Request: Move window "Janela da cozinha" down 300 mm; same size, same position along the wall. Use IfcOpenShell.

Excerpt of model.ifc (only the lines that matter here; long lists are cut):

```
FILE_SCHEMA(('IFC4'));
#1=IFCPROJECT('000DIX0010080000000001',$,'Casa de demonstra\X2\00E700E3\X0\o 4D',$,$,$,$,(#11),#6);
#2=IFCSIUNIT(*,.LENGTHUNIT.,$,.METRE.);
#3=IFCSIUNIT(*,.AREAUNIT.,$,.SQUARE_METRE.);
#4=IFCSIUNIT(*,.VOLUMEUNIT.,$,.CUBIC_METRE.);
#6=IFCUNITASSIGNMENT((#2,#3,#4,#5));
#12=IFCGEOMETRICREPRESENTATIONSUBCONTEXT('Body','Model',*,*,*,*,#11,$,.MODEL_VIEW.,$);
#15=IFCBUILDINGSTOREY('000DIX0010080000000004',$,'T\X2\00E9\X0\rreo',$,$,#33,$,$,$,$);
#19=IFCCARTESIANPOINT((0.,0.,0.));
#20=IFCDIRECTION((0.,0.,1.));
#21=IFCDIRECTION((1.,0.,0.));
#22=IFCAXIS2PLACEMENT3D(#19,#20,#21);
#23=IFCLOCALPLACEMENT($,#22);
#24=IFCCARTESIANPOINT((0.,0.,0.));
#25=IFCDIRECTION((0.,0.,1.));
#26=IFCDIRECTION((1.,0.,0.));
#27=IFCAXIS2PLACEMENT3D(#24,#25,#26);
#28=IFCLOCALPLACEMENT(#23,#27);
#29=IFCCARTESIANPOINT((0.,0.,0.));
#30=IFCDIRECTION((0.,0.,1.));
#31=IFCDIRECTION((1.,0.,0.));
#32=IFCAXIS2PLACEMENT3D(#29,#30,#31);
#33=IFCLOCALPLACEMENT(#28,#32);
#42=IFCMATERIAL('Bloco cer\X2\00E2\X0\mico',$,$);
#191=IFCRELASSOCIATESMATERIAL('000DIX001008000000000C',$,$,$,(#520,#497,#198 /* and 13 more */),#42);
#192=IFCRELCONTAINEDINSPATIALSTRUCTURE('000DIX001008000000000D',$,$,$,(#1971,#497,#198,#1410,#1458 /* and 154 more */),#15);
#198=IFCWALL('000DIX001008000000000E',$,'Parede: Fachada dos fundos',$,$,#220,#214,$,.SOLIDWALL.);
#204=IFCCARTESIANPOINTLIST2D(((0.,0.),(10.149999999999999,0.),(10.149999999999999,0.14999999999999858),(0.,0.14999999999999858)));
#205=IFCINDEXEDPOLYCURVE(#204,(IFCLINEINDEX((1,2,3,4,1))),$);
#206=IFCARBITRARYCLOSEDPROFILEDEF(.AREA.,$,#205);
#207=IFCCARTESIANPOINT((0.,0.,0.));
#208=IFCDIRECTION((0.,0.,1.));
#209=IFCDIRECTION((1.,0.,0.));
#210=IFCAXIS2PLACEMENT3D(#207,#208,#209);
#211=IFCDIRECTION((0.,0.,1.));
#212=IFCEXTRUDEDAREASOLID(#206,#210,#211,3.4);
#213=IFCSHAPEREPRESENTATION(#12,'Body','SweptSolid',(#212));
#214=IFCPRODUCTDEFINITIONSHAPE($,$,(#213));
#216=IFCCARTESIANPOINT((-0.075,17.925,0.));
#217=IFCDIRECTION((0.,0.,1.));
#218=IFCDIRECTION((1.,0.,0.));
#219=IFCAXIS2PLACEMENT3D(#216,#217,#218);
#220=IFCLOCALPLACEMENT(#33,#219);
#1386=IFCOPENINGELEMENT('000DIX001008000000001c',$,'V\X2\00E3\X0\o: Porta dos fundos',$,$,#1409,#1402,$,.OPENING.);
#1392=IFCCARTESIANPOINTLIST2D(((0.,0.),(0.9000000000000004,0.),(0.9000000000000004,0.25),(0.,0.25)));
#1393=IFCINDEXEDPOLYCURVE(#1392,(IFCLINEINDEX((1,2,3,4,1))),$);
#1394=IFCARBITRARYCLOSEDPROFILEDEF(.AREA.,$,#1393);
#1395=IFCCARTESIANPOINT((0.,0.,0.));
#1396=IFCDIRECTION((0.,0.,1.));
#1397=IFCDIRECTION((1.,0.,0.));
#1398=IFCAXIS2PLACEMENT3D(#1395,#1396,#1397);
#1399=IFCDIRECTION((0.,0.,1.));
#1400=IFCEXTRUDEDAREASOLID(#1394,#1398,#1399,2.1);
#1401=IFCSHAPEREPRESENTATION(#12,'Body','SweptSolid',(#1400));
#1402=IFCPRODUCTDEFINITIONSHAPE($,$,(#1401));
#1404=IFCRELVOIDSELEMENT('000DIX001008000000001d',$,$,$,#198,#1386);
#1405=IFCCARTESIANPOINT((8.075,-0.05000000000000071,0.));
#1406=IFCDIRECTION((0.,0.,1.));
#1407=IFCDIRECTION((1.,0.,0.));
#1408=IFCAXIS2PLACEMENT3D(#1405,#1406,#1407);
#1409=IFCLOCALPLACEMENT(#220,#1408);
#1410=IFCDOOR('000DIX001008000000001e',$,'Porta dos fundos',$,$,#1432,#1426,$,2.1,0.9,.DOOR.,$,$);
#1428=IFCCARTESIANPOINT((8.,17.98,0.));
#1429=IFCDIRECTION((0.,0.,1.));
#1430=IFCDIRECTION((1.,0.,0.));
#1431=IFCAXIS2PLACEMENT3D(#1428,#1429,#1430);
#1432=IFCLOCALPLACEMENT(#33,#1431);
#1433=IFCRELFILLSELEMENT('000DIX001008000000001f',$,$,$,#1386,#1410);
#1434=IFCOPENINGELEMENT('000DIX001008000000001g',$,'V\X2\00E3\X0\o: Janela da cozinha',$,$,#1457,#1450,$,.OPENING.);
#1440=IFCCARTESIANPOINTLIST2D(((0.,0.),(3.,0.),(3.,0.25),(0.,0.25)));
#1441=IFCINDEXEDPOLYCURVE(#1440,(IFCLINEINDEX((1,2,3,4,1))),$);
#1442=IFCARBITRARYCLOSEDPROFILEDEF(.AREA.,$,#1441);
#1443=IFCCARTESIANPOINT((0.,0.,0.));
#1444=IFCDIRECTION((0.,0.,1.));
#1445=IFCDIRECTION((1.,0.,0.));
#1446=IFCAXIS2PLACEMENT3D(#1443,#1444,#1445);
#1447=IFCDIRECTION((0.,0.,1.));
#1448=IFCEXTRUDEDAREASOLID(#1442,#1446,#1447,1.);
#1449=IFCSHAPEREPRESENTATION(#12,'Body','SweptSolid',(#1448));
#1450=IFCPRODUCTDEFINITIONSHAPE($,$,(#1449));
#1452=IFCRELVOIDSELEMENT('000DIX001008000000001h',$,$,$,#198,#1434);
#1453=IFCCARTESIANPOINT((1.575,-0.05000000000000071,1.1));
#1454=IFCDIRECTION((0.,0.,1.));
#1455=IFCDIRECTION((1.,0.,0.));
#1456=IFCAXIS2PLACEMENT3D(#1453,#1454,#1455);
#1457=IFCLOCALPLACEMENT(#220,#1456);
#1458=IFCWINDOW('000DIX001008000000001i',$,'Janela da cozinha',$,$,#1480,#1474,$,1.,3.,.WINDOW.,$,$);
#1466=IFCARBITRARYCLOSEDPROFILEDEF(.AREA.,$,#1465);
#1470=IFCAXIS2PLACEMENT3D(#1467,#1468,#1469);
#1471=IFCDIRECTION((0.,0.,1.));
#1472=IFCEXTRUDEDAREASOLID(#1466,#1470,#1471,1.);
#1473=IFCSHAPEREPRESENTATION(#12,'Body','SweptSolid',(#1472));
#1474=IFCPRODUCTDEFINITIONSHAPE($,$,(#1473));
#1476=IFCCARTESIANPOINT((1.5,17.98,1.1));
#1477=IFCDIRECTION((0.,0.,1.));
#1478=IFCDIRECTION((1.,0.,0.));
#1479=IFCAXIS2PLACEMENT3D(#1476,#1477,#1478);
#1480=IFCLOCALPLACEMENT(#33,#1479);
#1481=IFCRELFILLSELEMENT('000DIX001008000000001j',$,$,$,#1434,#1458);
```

```python
import numpy as np
import ifcopenshell
import ifcopenshell.api.geometry
import ifcopenshell.util.placement
import ifcopenshell.util.unit

model = ifcopenshell.open("model.ifc")
unit_scale = ifcopenshell.util.unit.calculate_unit_scale(model)

window = model.by_id(1458)
opening = window.FillsVoids[0].RelatingOpeningElement
dz = -0.3 / unit_scale

shift = np.array([0.0, 0.0, dz])
# The window is not placed relative to its opening, so move both.
for product in (opening, window):
    matrix = ifcopenshell.util.placement.get_local_placement(product.ObjectPlacement)
    matrix[:3, 3] += shift
    ifcopenshell.api.geometry.edit_object_placement(model, product=product, matrix=matrix, is_si=False)

print(f"moved by {dz * unit_scale:+.3f} m")

model.write("model_updated.ifc")
```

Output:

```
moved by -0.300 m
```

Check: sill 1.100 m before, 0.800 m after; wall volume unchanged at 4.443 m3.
